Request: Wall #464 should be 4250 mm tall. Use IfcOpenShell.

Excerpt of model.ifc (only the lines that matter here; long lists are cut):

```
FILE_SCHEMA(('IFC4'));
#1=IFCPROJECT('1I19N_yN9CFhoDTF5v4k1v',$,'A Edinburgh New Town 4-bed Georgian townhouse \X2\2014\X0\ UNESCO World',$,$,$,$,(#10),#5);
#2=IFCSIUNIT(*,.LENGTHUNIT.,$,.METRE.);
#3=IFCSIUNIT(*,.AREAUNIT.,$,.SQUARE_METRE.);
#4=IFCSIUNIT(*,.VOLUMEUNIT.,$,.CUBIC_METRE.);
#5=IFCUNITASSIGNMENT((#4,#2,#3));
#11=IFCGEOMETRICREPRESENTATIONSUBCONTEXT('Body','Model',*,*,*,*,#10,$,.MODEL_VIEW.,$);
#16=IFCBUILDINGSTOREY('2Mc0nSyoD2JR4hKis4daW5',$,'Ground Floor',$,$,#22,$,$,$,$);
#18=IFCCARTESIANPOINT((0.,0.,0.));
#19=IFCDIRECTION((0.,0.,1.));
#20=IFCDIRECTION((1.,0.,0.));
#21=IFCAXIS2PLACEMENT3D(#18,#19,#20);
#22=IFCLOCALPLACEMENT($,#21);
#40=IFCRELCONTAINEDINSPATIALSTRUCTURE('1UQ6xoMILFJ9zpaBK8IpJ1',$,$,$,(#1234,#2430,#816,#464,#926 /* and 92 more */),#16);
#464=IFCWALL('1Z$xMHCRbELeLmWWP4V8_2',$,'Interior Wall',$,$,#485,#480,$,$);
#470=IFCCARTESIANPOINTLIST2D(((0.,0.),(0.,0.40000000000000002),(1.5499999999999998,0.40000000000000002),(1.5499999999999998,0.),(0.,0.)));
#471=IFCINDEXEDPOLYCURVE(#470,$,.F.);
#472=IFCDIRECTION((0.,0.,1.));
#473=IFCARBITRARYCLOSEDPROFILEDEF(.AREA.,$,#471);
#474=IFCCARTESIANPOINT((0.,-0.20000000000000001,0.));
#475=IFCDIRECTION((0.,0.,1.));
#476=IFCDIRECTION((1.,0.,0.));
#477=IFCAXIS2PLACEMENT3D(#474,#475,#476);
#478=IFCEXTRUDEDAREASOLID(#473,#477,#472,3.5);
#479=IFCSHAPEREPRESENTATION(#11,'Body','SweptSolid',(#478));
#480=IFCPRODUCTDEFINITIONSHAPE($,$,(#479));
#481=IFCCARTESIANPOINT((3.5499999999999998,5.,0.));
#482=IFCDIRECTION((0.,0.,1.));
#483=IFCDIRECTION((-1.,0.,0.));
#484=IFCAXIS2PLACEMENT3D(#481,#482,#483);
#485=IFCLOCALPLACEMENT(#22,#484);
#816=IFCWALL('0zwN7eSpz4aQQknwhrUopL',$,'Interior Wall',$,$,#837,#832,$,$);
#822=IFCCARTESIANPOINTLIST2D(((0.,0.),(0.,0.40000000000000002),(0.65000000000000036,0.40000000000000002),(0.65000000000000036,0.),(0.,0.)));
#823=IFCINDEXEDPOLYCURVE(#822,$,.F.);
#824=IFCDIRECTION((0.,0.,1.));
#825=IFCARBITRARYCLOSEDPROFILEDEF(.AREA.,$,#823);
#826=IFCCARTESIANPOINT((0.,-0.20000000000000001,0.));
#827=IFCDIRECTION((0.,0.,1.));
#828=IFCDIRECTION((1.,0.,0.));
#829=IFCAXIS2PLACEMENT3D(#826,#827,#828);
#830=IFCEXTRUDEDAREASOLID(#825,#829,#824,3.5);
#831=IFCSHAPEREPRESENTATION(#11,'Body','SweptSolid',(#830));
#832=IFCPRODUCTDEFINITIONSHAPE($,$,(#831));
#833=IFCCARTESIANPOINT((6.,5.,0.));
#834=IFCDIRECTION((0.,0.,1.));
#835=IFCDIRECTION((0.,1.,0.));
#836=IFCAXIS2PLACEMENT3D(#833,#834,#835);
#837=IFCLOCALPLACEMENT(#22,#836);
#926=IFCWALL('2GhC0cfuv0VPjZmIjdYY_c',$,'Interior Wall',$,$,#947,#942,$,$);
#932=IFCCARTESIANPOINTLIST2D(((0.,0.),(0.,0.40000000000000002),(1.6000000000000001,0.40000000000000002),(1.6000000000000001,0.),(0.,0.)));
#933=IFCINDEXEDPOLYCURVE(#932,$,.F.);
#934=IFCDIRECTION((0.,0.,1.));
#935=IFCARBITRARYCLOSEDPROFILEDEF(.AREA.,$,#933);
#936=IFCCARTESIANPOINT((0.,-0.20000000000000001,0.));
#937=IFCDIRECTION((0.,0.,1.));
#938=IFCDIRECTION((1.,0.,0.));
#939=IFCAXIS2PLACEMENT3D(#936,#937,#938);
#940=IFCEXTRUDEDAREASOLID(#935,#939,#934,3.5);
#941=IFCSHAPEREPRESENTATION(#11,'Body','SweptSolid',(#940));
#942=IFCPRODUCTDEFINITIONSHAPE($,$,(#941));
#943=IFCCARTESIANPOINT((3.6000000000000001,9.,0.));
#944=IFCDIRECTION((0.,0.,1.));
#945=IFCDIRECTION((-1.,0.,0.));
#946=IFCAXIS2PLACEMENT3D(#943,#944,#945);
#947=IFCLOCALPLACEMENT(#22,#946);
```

```python
import ifcopenshell
import ifcopenshell.geom
import ifcopenshell.util.representation
import ifcopenshell.util.shape

model = ifcopenshell.open("model.ifc")
settings = ifcopenshell.geom.settings()


def volume(element):
    """Net volume in cubic metres, openings subtracted."""
    shape = ifcopenshell.geom.create_shape(settings, element)
    return ifcopenshell.util.shape.get_volume(shape.geometry)


wall = model.by_id(464)
before = volume(wall)

body = ifcopenshell.util.representation.get_representation(wall, "Model", "Body")
solid = body.Items[0]
old_height = solid.Depth
solid.Depth = 4.25
after = volume(wall)

print(f"height {old_height:g} -> {solid.Depth:g}, volume {before:.3f} -> {after:.3f} m3")

model.write("model-out.ifc")
```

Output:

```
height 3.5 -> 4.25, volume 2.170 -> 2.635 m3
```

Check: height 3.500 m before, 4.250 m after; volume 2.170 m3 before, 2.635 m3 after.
